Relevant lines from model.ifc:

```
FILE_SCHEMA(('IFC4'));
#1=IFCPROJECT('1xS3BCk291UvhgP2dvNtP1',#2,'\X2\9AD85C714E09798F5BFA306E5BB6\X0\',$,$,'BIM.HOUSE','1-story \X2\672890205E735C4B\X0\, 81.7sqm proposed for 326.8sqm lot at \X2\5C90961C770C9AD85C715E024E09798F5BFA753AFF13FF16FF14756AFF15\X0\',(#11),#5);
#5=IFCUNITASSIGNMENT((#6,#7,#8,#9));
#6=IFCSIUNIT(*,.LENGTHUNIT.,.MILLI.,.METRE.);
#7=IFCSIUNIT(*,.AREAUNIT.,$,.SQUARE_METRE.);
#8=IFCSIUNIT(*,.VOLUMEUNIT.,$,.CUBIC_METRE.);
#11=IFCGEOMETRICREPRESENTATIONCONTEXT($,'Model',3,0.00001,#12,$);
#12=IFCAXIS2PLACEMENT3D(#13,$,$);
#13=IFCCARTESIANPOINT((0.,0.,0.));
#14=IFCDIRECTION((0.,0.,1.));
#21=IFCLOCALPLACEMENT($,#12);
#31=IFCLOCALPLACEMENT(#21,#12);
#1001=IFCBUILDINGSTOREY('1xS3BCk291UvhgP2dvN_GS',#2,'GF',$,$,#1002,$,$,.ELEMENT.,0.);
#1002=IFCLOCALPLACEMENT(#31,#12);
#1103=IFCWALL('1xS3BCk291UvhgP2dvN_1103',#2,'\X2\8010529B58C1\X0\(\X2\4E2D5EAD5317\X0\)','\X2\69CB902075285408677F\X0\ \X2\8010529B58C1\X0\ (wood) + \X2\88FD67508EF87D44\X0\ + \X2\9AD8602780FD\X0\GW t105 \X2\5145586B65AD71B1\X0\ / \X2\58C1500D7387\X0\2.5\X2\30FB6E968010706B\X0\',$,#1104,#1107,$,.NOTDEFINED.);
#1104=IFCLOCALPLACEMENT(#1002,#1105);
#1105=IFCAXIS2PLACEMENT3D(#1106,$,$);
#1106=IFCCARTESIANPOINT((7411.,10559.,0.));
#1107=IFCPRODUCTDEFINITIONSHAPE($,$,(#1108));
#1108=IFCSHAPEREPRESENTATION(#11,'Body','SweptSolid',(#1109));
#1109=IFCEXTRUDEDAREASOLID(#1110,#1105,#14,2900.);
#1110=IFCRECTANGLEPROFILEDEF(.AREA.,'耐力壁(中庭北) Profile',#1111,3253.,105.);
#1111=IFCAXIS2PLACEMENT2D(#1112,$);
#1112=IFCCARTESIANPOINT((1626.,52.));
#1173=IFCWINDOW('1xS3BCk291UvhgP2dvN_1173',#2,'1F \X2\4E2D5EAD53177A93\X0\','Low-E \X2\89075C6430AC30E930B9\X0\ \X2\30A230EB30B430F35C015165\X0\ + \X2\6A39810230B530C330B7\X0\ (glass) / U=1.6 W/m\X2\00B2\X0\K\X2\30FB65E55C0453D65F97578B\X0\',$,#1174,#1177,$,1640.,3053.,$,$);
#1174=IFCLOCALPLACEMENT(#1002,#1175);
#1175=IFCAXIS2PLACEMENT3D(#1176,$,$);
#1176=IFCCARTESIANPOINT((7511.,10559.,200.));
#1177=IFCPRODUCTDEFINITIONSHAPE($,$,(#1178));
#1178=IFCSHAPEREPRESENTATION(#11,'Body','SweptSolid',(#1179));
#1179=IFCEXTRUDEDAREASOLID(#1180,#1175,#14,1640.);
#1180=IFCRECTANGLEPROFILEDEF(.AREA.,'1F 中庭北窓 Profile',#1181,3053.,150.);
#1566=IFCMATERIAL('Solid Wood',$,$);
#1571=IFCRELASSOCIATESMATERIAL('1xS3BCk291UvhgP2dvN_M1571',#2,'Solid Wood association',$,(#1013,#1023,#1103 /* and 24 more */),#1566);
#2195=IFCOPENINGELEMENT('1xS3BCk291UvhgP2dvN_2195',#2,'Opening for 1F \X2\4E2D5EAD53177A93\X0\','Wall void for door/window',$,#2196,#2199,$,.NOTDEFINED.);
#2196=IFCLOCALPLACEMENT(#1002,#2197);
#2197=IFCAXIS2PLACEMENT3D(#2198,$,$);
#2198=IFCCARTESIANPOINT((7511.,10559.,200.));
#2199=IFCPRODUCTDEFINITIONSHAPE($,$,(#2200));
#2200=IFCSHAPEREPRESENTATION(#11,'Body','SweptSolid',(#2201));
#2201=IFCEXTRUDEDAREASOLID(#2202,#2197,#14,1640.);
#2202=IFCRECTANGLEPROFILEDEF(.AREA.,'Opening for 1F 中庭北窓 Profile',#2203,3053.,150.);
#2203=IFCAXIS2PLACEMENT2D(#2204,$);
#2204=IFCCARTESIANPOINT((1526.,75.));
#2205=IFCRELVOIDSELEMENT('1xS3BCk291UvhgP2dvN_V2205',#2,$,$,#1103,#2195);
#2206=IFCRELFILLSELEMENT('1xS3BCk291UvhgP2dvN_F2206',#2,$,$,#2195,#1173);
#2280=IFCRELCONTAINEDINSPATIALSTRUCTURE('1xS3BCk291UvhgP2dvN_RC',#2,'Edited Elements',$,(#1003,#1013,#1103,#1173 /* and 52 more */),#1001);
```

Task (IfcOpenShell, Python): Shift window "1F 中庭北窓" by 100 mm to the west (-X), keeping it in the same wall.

```python
import ifcopenshell
import ifcopenshell.api.geometry
import ifcopenshell.util.placement

model = ifcopenshell.open("model.ifc")

window = model.by_id(1173)
opening = window.FillsVoids[0].RelatingOpeningElement
wall = opening.VoidsElements[0].RelatingBuildingElement

wall_matrix = ifcopenshell.util.placement.get_local_placement(wall.ObjectPlacement)
shift = wall_matrix[:3, 0] * -100.0
before = ifcopenshell.util.placement.get_local_placement(window.ObjectPlacement)[:3, 3].copy()

# The window is not placed relative to its opening, so move both.
for product in (opening, window):
    matrix = ifcopenshell.util.placement.get_local_placement(product.ObjectPlacement)
    matrix[:3, 3] += shift
    ifcopenshell.api.geometry.edit_object_placement(model, product=product, matrix=matrix, is_si=False)

after = ifcopenshell.util.placement.get_local_placement(window.ObjectPlacement)[:3, 3]
print("window moved by", (after - before).round(3) + 0.0)

model.write("model-out.ifc")
```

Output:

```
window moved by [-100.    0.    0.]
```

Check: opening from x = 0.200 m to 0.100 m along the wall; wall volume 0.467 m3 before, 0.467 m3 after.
